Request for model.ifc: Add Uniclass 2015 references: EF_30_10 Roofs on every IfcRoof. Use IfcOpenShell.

First a look at what the model holds.

```python
import ifcopenshell

model = ifcopenshell.open("model.ifc")
print(model.schema)
print("classifications:", [c.Name for c in model.by_type("IfcClassification")])
for ifc_class in ("IfcDoor", "IfcRoof", "IfcStair", "IfcWall", "IfcWindow"):
    print(ifc_class, len(model.by_type(ifc_class)))
```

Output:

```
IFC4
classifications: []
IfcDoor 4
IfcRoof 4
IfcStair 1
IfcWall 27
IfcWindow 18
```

```python
import ifcopenshell
import ifcopenshell.api.classification

model = ifcopenshell.open("model.ifc")

system = ifcopenshell.api.classification.add_classification(model, classification="Uniclass 2015")

codes = {
    "IfcRoof": ("EF_30_10", "Roofs"),
}
for ifc_class, (code, name) in codes.items():
    products = model.by_type(ifc_class)
    ifcopenshell.api.classification.add_reference(
        model, products=products, classification=system, identification=code, name=name
    )
    print(code, len(products))

model.write("model_v2.ifc")
```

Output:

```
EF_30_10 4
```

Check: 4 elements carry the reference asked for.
